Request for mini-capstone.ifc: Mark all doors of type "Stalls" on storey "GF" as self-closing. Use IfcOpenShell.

First a look at what the model holds.

```python
import ifcopenshell
import ifcopenshell.util.element

model = ifcopenshell.open("mini-capstone.ifc")
print(model.schema)
storey = next(s for s in model.by_type("IfcBuildingStorey") if s.Name == "GF")
doors = [e for e in ifcopenshell.util.element.get_decomposition(storey) if e.is_a("IfcDoor")]
seen = {}
for e in doors:
    element_type = ifcopenshell.util.element.get_type(e)
    key = (element_type.Name if element_type != e and element_type else None, ifcopenshell.util.element.get_pset(e, "Pset_DoorCommon", "SelfClosing"))
    seen[key] = seen.get(key, 0) + 1
for (name, value), count in sorted(seen.items(), key=str):
    print(count, "x", name, "|", value)
```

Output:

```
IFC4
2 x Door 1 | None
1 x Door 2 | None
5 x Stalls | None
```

```python
import ifcopenshell
import ifcopenshell.api.pset
import ifcopenshell.util.element

model = ifcopenshell.open("mini-capstone.ifc")

storey = next(s for s in model.by_type("IfcBuildingStorey") if s.Name == "GF")
doors = [e for e in ifcopenshell.util.element.get_decomposition(storey) if e.is_a("IfcDoor")]

count = 0
for e in doors:
    element_type = ifcopenshell.util.element.get_type(e)
    if element_type in (None, e) or element_type.Name != "Stalls":
        continue
    # add_pset returns the element's existing set when there is one.
    pset = ifcopenshell.api.pset.add_pset(model, product=e, name="Pset_DoorCommon")
    ifcopenshell.api.pset.edit_pset(model, pset=pset, properties={"SelfClosing": True})
    count += 1

print(count, "doors updated")

model.write("mini-capstone_edited.ifc")
```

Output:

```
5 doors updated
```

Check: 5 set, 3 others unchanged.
